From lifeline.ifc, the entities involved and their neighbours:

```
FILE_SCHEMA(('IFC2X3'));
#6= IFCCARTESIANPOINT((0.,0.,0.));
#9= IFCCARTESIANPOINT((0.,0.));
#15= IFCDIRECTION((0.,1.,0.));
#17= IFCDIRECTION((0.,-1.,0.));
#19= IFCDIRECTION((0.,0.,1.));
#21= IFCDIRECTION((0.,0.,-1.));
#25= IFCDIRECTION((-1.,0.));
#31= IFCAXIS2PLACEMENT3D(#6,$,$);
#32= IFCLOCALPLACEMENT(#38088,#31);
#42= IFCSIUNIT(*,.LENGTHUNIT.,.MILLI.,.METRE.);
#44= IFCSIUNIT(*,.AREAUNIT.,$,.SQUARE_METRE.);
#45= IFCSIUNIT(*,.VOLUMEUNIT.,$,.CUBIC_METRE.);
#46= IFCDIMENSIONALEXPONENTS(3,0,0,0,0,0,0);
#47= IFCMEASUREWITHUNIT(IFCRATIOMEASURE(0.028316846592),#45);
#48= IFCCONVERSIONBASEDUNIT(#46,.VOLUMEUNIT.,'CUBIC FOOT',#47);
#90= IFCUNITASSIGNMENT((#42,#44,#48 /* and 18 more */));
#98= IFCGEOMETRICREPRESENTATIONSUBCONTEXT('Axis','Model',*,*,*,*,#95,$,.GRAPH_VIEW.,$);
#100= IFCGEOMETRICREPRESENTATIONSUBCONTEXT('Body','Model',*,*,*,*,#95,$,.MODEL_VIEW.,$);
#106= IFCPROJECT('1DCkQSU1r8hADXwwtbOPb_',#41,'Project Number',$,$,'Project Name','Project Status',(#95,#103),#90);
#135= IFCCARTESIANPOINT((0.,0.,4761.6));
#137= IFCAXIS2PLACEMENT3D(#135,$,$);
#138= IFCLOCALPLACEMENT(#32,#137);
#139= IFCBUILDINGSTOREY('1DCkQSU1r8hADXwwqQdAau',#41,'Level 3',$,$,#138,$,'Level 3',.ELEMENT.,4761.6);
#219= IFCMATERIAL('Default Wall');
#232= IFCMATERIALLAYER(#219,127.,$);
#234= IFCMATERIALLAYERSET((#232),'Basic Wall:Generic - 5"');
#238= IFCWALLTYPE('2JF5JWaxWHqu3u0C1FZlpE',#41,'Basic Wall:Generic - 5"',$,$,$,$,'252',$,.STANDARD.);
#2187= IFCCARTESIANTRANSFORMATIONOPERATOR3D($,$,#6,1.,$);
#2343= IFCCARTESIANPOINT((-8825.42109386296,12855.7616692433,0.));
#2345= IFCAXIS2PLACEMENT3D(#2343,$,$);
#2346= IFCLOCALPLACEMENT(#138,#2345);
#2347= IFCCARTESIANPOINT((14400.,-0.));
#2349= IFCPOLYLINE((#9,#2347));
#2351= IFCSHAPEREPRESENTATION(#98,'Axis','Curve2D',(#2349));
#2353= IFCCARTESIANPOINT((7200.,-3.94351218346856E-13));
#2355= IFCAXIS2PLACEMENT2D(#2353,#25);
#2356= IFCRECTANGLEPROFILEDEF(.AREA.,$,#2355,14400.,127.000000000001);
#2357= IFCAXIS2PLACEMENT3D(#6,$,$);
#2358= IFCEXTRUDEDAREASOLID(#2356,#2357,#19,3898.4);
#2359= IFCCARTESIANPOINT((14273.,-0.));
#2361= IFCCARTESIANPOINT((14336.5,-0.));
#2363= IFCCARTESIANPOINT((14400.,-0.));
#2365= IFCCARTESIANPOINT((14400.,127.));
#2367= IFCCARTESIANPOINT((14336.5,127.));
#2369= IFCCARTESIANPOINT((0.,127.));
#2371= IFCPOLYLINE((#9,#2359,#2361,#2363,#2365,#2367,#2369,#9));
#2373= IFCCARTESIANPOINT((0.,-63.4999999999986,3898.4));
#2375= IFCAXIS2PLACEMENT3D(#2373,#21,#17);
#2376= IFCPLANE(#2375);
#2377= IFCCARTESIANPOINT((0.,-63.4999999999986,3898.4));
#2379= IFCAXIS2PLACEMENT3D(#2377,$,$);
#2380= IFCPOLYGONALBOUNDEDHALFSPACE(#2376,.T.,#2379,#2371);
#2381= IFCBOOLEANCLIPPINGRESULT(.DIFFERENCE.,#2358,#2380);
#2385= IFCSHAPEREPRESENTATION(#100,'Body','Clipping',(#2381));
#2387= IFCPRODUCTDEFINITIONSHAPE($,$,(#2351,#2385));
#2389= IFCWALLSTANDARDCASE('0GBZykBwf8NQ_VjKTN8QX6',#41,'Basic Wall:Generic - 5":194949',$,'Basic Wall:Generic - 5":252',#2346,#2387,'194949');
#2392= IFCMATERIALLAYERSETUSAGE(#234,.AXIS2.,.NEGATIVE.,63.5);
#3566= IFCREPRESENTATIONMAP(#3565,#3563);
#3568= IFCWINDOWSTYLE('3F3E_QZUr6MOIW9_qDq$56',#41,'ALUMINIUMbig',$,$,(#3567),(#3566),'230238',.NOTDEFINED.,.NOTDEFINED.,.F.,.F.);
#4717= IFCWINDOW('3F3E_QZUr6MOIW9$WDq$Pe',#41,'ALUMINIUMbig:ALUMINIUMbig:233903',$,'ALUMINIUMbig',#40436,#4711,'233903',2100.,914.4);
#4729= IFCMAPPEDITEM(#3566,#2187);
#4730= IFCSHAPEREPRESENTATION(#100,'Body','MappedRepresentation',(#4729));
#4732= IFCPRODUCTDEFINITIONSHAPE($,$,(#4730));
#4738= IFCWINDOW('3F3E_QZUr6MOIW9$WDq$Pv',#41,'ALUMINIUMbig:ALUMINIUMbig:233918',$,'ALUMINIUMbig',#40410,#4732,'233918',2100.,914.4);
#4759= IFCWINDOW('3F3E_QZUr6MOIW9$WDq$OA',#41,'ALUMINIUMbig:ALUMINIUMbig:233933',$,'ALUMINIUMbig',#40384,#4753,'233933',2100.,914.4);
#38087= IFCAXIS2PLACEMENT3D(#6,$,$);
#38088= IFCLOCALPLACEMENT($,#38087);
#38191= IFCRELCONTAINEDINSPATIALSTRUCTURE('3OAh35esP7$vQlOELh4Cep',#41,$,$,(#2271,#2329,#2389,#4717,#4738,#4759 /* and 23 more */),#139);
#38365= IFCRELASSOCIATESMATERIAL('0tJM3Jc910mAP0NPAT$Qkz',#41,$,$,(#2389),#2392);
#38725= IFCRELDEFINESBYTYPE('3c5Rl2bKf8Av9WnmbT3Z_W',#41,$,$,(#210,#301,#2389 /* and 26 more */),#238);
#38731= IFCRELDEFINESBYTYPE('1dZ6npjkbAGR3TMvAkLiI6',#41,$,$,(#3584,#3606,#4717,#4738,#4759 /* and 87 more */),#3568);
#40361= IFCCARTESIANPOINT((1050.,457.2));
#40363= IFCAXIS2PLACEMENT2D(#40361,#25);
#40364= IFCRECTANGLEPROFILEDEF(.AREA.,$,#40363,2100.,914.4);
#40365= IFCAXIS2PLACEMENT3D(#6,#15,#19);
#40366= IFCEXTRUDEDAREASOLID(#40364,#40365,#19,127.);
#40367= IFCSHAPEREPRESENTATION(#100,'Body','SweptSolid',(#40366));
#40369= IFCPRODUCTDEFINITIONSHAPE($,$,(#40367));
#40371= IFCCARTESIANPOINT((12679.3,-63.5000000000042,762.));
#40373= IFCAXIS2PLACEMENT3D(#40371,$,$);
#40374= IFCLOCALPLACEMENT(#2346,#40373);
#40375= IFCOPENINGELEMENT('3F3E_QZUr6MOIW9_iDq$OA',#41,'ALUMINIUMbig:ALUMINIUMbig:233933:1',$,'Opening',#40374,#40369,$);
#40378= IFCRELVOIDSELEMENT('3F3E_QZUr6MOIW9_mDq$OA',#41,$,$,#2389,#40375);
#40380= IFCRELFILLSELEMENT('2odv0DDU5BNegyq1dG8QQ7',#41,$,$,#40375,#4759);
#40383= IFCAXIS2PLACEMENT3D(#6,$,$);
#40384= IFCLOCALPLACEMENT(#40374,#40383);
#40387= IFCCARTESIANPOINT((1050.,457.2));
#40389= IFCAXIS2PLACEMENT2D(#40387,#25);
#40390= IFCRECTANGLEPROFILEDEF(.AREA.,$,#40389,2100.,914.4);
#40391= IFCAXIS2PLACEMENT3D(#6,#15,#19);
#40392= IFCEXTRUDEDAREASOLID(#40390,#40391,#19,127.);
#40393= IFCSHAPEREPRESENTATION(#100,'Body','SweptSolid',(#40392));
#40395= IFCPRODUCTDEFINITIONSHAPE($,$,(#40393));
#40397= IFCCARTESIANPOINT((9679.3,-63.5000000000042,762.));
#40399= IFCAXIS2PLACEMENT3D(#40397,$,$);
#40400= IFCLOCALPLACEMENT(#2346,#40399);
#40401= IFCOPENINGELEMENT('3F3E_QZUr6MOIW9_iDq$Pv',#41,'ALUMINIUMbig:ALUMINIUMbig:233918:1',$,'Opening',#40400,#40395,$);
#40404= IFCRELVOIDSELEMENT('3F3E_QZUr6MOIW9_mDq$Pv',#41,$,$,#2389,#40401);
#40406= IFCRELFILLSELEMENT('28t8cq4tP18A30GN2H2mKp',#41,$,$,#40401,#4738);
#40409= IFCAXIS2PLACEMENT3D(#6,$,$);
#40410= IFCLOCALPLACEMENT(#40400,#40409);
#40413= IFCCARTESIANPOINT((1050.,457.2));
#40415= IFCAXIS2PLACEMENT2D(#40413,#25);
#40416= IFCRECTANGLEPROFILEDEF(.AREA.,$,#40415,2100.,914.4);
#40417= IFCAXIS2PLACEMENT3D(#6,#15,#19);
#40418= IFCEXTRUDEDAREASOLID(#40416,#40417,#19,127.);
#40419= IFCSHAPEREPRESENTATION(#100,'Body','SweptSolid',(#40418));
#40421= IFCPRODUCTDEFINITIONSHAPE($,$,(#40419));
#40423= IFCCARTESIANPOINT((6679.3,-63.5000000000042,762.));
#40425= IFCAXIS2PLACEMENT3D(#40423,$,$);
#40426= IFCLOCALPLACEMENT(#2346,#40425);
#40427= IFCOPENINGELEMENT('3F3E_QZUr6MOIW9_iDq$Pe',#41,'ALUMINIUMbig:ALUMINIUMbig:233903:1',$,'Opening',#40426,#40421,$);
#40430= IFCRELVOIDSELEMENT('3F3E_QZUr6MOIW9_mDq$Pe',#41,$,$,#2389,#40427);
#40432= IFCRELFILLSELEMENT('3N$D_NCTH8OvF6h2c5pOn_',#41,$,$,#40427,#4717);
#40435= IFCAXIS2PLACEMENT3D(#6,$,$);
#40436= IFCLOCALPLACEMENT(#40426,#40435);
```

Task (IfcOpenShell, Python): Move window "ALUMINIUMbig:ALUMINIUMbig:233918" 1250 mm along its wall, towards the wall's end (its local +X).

```python
import ifcopenshell
import ifcopenshell.api.geometry
import ifcopenshell.util.placement

model = ifcopenshell.open("lifeline.ifc")

window = model.by_guid("3F3E_QZUr6MOIW9$WDq$Pv")
opening = window.FillsVoids[0].RelatingOpeningElement
wall = opening.VoidsElements[0].RelatingBuildingElement

wall_matrix = ifcopenshell.util.placement.get_local_placement(wall.ObjectPlacement)
shift = wall_matrix[:3, 0] * 1250.0
before = ifcopenshell.util.placement.get_local_placement(window.ObjectPlacement)[:3, 3].copy()

# The window is placed relative to its opening, so it follows when the opening moves.
matrix = ifcopenshell.util.placement.get_local_placement(opening.ObjectPlacement)
matrix[:3, 3] += shift
ifcopenshell.api.geometry.edit_object_placement(
    model, product=opening, matrix=matrix, is_si=False, should_transform_children=True
)

after = ifcopenshell.util.placement.get_local_placement(window.ObjectPlacement)[:3, 3]
print("window moved by", (after - before).round(3) + 0.0)

model.write("lifeline_rev.ifc")
```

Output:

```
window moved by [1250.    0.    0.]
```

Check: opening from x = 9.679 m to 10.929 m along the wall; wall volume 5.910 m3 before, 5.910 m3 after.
